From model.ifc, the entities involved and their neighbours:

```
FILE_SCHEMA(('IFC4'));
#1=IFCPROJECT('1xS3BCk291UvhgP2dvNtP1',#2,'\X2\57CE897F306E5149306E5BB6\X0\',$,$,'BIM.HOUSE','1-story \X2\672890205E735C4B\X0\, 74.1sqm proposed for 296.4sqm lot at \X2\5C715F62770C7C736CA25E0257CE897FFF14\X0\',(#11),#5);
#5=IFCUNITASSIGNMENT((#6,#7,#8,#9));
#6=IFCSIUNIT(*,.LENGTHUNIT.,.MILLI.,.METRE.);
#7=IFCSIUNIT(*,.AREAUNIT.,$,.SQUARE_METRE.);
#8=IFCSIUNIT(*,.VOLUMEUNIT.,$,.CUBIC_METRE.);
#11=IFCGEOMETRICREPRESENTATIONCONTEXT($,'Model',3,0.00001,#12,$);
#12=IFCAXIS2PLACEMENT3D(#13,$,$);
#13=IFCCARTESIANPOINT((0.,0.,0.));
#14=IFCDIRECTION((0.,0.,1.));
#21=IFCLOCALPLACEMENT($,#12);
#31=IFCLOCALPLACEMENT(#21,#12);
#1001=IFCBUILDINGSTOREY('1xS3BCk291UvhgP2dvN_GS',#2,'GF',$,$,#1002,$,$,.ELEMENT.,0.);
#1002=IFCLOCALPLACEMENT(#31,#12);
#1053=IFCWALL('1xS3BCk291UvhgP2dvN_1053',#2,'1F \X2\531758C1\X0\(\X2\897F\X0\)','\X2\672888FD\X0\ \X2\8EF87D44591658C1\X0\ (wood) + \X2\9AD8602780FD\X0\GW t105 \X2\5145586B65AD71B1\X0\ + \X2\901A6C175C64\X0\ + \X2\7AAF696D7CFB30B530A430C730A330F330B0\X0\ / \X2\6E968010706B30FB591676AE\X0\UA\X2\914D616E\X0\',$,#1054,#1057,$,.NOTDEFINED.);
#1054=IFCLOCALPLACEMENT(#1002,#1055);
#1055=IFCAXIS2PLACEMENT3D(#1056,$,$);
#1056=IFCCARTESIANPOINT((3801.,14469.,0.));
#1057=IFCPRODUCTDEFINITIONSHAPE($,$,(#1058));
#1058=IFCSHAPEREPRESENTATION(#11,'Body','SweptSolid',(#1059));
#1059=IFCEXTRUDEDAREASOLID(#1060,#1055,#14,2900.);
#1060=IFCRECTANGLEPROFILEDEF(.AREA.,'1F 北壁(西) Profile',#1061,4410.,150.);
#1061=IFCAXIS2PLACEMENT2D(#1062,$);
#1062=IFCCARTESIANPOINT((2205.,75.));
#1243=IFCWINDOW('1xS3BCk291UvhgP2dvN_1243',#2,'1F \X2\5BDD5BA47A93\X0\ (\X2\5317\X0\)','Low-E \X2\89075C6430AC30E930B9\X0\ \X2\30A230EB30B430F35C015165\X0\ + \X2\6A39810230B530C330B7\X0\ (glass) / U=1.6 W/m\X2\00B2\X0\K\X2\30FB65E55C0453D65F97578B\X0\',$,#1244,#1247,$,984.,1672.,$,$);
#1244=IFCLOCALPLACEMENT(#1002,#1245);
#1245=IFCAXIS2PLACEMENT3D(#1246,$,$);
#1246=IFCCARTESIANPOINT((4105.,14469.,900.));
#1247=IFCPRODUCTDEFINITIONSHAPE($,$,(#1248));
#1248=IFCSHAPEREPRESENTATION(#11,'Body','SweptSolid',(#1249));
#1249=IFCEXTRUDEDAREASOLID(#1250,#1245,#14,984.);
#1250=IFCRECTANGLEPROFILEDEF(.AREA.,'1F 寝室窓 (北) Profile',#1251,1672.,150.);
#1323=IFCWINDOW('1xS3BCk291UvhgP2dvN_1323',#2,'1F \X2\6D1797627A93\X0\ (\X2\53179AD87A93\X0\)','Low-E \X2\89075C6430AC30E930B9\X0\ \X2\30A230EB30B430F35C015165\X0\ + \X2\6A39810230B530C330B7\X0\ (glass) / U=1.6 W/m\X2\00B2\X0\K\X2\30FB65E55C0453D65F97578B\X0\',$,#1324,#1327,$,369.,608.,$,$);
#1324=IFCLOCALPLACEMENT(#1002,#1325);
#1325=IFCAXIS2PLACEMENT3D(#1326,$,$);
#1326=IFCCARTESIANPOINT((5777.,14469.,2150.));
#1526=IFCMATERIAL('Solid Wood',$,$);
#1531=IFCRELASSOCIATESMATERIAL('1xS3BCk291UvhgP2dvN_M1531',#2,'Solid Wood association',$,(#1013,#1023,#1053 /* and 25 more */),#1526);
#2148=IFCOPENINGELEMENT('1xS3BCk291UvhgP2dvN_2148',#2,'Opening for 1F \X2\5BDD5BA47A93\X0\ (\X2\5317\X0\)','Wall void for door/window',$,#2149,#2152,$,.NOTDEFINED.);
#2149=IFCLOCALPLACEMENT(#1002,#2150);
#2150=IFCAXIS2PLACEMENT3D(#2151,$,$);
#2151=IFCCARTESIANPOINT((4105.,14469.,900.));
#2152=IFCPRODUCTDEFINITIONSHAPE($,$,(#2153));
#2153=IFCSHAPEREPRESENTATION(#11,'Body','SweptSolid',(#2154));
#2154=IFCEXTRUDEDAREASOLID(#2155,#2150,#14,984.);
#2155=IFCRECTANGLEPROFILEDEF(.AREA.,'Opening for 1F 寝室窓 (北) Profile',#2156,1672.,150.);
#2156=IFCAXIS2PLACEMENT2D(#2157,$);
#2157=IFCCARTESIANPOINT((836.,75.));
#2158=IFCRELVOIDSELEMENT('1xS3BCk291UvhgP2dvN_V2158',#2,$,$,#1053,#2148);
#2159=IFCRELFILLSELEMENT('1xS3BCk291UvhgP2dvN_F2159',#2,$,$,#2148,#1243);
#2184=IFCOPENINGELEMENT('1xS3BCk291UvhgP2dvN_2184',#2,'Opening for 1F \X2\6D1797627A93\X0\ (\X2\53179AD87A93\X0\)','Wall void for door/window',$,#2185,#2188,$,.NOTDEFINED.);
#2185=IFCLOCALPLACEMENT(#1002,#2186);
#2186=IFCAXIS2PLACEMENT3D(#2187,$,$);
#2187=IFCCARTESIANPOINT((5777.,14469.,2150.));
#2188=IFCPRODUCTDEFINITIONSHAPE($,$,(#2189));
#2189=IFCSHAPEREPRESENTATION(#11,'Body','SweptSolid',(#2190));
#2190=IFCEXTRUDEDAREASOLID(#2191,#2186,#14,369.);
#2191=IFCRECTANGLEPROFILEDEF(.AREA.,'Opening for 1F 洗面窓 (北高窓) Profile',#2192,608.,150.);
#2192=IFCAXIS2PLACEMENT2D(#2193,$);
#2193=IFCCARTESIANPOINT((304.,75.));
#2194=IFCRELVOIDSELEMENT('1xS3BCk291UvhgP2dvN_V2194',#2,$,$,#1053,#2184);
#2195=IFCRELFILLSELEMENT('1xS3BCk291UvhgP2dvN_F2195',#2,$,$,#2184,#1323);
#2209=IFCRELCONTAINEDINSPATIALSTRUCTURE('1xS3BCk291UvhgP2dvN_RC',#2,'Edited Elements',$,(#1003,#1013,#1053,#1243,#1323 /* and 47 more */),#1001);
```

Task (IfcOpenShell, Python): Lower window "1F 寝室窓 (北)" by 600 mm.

```python
import numpy as np
import ifcopenshell
import ifcopenshell.api.geometry
import ifcopenshell.util.placement
import ifcopenshell.util.unit

model = ifcopenshell.open("model.ifc")
unit_scale = ifcopenshell.util.unit.calculate_unit_scale(model)

window = model.by_id(1243)
opening = window.FillsVoids[0].RelatingOpeningElement
dz = -0.6 / unit_scale

shift = np.array([0.0, 0.0, dz])
# The window is not placed relative to its opening, so move both.
for product in (opening, window):
    matrix = ifcopenshell.util.placement.get_local_placement(product.ObjectPlacement)
    matrix[:3, 3] += shift
    ifcopenshell.api.geometry.edit_object_placement(model, product=product, matrix=matrix, is_si=False)

print(f"moved by {dz * unit_scale:+.3f} m")

model.write("model_rev.ifc")
```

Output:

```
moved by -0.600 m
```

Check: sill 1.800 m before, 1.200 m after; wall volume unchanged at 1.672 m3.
